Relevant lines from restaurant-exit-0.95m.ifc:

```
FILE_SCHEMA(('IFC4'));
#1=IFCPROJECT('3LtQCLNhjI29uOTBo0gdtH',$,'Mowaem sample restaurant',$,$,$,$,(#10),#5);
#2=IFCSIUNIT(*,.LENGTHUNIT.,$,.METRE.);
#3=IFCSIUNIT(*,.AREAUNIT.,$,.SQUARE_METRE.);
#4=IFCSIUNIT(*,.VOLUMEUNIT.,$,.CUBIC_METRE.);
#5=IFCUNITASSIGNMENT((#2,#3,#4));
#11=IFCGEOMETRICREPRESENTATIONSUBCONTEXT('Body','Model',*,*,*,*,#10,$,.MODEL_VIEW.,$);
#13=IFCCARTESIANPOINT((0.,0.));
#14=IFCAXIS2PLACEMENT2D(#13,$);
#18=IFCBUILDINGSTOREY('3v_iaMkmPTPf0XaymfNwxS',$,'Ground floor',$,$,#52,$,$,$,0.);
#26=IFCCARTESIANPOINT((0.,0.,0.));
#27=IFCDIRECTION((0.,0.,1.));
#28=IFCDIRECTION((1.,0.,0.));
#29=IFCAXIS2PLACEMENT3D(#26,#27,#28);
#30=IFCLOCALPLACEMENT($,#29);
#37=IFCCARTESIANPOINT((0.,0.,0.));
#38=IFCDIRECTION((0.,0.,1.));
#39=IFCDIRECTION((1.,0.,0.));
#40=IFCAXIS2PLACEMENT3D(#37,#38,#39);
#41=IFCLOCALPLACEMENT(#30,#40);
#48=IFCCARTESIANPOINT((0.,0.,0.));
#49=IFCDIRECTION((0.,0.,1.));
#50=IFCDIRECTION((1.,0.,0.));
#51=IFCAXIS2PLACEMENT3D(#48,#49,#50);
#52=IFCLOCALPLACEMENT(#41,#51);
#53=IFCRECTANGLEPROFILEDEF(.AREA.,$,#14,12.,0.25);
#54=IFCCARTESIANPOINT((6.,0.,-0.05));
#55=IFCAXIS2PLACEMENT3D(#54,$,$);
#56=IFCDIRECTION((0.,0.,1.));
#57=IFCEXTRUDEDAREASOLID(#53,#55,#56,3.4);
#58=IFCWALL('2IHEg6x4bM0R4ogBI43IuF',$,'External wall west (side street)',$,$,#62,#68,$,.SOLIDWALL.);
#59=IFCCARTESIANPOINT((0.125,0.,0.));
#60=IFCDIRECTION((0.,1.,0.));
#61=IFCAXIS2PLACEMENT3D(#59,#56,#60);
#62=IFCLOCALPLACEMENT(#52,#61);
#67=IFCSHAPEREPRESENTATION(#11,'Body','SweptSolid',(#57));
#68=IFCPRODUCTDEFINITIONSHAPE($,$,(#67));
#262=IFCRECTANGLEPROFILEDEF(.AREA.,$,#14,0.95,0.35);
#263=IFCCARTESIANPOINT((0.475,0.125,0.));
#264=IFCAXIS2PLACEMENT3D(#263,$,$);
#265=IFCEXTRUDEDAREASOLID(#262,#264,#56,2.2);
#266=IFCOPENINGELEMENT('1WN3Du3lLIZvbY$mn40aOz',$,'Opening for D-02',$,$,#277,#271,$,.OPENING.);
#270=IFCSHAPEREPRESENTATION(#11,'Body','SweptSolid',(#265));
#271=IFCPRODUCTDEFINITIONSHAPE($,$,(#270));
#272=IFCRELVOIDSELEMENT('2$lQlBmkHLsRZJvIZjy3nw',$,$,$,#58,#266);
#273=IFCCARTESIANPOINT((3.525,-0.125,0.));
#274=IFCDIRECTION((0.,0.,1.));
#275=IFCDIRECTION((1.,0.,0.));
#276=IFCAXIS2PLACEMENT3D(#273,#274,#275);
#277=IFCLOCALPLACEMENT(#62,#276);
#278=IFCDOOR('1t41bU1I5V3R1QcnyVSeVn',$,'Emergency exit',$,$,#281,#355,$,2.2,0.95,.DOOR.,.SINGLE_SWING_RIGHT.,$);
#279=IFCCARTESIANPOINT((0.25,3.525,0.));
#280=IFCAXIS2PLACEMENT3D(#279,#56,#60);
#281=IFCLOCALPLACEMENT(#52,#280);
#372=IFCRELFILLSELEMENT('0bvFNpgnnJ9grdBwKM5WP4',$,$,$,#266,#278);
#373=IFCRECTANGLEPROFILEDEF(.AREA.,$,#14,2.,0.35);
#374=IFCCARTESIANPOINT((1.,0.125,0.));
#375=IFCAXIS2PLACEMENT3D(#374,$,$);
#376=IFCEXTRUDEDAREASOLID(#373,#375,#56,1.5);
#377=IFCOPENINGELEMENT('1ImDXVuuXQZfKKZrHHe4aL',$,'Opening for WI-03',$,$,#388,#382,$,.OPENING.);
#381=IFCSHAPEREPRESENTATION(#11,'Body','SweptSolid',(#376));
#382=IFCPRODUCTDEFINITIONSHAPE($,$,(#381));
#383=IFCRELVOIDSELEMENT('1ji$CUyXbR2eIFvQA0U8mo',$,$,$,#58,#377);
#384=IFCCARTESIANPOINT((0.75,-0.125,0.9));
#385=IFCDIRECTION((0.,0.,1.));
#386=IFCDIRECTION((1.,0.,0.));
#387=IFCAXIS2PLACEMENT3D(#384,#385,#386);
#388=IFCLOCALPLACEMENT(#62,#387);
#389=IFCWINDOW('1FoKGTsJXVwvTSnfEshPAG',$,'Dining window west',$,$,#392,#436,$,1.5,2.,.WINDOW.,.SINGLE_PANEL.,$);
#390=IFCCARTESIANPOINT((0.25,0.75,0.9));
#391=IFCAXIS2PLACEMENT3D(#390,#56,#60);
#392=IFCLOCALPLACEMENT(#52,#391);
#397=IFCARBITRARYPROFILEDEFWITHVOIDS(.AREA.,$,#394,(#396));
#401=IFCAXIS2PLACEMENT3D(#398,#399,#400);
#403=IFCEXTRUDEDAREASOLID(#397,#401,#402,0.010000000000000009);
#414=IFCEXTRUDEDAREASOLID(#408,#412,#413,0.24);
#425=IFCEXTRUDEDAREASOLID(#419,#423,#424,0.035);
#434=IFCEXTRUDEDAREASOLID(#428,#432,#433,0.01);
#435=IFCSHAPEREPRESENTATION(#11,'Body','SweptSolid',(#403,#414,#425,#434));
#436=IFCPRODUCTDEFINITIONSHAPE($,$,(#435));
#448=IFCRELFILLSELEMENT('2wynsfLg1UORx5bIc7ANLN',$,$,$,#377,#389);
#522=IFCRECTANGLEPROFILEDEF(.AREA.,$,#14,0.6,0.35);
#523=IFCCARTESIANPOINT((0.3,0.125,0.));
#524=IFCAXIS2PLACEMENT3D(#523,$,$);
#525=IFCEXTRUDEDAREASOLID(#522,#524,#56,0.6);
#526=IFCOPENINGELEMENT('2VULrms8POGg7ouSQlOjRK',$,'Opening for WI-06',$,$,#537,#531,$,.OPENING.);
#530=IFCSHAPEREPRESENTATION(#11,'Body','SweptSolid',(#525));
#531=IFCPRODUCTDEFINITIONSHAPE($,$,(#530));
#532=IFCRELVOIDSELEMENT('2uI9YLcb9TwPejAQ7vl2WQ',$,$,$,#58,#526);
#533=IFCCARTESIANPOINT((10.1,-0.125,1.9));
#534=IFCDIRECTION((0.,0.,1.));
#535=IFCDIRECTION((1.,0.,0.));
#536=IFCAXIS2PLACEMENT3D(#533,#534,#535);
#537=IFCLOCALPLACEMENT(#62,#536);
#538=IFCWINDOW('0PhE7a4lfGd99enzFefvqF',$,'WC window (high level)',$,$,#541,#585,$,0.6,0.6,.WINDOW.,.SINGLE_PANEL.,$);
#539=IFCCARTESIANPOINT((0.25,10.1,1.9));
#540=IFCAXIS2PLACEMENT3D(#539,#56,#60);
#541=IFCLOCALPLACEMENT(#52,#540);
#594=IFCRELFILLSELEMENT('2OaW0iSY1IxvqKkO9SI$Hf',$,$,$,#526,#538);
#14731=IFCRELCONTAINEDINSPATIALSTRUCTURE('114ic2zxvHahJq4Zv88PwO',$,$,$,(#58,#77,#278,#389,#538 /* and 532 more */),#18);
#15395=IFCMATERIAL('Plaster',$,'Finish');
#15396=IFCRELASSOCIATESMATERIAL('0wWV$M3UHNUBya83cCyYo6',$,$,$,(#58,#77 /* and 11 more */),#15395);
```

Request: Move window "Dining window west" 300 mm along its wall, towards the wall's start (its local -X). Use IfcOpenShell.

```python
import ifcopenshell
import ifcopenshell.api.geometry
import ifcopenshell.util.placement
import ifcopenshell.util.unit

model = ifcopenshell.open("restaurant-exit-0.95m.ifc")
unit_scale = ifcopenshell.util.unit.calculate_unit_scale(model)

window = model.by_id(389)
opening = window.FillsVoids[0].RelatingOpeningElement
wall = opening.VoidsElements[0].RelatingBuildingElement

wall_matrix = ifcopenshell.util.placement.get_local_placement(wall.ObjectPlacement)
shift = wall_matrix[:3, 0] * -0.3 / unit_scale
before = ifcopenshell.util.placement.get_local_placement(window.ObjectPlacement)[:3, 3].copy()

# The window is not placed relative to its opening, so move both.
for product in (opening, window):
    matrix = ifcopenshell.util.placement.get_local_placement(product.ObjectPlacement)
    matrix[:3, 3] += shift
    ifcopenshell.api.geometry.edit_object_placement(model, product=product, matrix=matrix, is_si=False)

after = ifcopenshell.util.placement.get_local_placement(window.ObjectPlacement)[:3, 3]
print("window moved by", (after - before).round(3) + 0.0)

model.write("restaurant-exit-0.95m_updated.ifc")
```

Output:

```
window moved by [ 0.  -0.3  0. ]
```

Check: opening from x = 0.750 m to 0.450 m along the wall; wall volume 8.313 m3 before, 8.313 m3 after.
